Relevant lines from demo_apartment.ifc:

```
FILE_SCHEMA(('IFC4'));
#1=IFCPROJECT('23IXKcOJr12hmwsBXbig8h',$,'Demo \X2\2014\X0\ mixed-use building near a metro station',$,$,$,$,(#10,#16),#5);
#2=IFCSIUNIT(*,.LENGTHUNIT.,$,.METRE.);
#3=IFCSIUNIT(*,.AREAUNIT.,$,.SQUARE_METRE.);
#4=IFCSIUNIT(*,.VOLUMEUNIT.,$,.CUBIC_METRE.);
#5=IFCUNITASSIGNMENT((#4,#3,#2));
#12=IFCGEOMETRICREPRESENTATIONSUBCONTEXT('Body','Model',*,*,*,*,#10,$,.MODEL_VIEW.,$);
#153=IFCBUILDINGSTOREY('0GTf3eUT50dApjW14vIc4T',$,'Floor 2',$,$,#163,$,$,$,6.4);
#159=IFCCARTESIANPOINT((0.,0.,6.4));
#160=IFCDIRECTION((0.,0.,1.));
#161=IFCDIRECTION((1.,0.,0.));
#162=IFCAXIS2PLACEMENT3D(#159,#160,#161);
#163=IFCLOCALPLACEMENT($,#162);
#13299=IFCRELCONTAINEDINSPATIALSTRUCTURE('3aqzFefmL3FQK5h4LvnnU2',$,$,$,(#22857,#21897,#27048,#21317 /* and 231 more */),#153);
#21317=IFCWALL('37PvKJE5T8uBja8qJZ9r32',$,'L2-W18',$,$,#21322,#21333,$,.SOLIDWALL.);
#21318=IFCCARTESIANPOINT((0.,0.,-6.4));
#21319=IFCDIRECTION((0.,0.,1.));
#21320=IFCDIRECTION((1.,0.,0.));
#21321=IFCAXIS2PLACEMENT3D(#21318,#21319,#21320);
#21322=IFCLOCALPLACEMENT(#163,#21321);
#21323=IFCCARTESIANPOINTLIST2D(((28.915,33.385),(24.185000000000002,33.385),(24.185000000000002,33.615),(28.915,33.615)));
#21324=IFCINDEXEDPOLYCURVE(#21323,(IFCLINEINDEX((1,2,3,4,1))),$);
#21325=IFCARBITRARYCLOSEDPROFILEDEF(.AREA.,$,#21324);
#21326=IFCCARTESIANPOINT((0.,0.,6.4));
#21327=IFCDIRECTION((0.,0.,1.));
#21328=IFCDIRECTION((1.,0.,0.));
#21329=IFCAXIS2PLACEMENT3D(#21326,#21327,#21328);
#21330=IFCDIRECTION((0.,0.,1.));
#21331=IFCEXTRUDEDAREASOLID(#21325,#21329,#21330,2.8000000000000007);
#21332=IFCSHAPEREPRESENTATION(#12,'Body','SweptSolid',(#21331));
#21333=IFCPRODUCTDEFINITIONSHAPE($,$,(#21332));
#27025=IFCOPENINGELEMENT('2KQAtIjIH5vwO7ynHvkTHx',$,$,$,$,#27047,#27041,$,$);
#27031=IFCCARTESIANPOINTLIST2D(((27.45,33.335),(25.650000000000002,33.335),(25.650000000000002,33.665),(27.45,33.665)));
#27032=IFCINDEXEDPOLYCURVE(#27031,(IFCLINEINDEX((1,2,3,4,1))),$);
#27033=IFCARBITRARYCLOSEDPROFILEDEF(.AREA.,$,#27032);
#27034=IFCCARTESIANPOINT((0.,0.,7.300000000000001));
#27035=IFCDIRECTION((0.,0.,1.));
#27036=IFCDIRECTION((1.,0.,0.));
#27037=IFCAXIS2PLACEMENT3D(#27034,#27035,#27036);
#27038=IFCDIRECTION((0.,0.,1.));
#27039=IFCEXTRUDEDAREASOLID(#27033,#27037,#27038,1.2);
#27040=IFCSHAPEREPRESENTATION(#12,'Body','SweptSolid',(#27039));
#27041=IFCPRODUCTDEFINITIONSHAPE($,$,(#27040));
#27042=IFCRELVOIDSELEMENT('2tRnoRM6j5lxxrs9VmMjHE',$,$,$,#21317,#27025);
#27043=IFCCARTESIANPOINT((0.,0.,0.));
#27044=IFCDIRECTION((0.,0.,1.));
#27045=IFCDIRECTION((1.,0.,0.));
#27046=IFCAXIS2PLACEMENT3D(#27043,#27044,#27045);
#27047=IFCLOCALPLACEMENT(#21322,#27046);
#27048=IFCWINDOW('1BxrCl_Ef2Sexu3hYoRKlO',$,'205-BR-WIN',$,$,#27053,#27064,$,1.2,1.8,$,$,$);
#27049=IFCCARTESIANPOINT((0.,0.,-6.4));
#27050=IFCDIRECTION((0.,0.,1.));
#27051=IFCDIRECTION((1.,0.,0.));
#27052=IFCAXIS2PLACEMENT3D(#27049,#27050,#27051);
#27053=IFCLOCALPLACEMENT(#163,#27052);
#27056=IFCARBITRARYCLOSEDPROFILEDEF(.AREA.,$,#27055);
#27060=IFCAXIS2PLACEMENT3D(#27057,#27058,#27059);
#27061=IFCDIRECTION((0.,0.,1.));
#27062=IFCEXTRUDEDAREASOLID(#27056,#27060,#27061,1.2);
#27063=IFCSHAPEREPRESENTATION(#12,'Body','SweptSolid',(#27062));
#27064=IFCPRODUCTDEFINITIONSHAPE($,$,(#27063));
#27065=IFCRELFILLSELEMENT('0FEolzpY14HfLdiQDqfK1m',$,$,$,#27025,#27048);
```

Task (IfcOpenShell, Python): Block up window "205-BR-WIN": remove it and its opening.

```python
import ifcopenshell
import ifcopenshell.api.feature
import ifcopenshell.api.root
import ifcopenshell.geom
import ifcopenshell.util.shape

model = ifcopenshell.open("demo_apartment.ifc")
settings = ifcopenshell.geom.settings()


def volume(element):
    """Net volume in cubic metres, openings subtracted."""
    shape = ifcopenshell.geom.create_shape(settings, element)
    return ifcopenshell.util.shape.get_volume(shape.geometry)


window = model.by_id(27048)
opening = window.FillsVoids[0].RelatingOpeningElement
wall = opening.VoidsElements[0].RelatingBuildingElement
before = volume(wall)

ifcopenshell.api.root.remove_product(model, product=window)
ifcopenshell.api.feature.remove_feature(model, feature=opening)

after = volume(wall)

print(f"wall volume {before:.3f} -> {after:.3f} m3")

model.write("demo_apartment_rev.ifc")
```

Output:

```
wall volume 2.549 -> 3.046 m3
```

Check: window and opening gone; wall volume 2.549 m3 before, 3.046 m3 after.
